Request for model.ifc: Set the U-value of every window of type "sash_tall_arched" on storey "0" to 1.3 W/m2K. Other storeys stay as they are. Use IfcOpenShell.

First a look at what the model holds.

```python
import ifcopenshell
import ifcopenshell.util.element

model = ifcopenshell.open("model.ifc")
print(model.schema)
storey = next(s for s in model.by_type("IfcBuildingStorey") if s.Name == "0")
windows = [e for e in ifcopenshell.util.element.get_decomposition(storey) if e.is_a("IfcWindow")]
seen = {}
for e in windows:
    element_type = ifcopenshell.util.element.get_type(e)
    key = (element_type.Name if element_type != e and element_type else None, ifcopenshell.util.element.get_pset(e, "Pset_WindowCommon", "ThermalTransmittance"))
    seen[key] = seen.get(key, 0) + 1
for (name, value), count in sorted(seen.items(), key=str):
    print(count, "x", name, "|", value)
```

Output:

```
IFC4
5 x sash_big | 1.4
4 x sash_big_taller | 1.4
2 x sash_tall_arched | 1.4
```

```python
import ifcopenshell
import ifcopenshell.api.pset
import ifcopenshell.util.element

model = ifcopenshell.open("model.ifc")

storey = next(s for s in model.by_type("IfcBuildingStorey") if s.Name == "0")
windows = [e for e in ifcopenshell.util.element.get_decomposition(storey) if e.is_a("IfcWindow")]

count = 0
for e in windows:
    element_type = ifcopenshell.util.element.get_type(e)
    if element_type in (None, e) or element_type.Name != "sash_tall_arched":
        continue
    # add_pset returns the element's existing set when there is one.
    pset = ifcopenshell.api.pset.add_pset(model, product=e, name="Pset_WindowCommon")
    ifcopenshell.api.pset.edit_pset(model, pset=pset, properties={"ThermalTransmittance": 1.3})
    count += 1

print(count, "windows updated")

model.write("model-out.ifc")
```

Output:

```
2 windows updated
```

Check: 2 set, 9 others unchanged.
